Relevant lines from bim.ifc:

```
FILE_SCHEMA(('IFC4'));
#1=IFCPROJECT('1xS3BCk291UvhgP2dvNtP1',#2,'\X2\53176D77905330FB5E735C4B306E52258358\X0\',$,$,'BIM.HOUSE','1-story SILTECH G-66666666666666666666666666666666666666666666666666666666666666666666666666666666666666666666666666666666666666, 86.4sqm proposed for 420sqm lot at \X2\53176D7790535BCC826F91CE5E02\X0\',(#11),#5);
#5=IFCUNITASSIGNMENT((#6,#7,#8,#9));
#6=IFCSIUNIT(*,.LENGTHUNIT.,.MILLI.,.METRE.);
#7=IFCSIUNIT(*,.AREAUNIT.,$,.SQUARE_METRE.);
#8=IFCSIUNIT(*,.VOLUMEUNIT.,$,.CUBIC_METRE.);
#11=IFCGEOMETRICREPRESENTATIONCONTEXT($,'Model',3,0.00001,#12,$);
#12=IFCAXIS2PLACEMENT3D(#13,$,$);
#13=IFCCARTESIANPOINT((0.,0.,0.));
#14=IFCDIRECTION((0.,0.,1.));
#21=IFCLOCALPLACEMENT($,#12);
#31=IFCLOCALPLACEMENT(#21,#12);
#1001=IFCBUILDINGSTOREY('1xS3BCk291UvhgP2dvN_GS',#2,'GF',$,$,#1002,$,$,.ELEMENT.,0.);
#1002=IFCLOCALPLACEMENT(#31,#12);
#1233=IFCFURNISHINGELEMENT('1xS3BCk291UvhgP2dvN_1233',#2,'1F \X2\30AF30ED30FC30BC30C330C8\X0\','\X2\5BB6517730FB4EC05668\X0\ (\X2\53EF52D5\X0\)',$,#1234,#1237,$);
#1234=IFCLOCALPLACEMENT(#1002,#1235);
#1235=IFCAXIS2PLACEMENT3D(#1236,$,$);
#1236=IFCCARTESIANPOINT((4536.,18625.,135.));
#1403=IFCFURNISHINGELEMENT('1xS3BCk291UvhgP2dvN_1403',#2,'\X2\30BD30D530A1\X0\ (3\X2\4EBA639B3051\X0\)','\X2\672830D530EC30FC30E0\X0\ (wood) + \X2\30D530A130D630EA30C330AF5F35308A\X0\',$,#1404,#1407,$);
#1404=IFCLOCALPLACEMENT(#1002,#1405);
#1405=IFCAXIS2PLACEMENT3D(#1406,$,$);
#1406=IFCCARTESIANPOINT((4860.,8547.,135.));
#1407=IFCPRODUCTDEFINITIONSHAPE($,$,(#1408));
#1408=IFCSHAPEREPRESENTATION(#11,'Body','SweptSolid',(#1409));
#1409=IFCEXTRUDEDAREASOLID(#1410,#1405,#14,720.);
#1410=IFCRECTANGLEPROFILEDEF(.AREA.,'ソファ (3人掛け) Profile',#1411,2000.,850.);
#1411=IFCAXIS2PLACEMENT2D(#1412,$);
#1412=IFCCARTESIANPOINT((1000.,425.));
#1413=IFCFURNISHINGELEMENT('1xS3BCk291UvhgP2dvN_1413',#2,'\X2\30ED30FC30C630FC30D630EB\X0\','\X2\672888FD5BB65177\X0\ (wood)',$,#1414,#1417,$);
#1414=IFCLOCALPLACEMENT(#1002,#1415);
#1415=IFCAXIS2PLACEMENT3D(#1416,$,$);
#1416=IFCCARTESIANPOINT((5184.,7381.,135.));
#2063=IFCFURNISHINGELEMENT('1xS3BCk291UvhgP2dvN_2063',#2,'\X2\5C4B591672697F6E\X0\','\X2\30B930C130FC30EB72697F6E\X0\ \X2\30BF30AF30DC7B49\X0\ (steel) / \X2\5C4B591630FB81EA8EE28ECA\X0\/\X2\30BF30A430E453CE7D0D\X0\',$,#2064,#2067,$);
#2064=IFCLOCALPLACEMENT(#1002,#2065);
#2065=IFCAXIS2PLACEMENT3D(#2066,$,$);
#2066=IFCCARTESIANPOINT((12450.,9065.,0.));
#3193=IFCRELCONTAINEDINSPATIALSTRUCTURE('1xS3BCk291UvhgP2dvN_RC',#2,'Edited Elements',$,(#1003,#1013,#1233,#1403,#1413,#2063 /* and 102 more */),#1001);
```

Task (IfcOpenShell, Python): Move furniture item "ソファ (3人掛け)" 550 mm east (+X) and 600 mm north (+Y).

```python
import ifcopenshell
import ifcopenshell.api.geometry
import ifcopenshell.util.placement
import ifcopenshell.util.unit

model = ifcopenshell.open("bim.ifc")
unit_scale = ifcopenshell.util.unit.calculate_unit_scale(model)

item = model.by_id(1403)
matrix = ifcopenshell.util.placement.get_local_placement(item.ObjectPlacement)
matrix[0, 3] += 0.55 / unit_scale
matrix[1, 3] += 0.6 / unit_scale
ifcopenshell.api.geometry.edit_object_placement(model, product=item, matrix=matrix, is_si=False)

print(ifcopenshell.util.placement.get_local_placement(item.ObjectPlacement).round(3) + 0.0)

model.write("bim_rev.ifc")
```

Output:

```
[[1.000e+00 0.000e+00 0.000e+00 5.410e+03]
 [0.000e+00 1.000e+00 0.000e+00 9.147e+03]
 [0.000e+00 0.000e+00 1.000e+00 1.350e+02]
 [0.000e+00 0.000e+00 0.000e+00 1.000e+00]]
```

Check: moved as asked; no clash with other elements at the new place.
